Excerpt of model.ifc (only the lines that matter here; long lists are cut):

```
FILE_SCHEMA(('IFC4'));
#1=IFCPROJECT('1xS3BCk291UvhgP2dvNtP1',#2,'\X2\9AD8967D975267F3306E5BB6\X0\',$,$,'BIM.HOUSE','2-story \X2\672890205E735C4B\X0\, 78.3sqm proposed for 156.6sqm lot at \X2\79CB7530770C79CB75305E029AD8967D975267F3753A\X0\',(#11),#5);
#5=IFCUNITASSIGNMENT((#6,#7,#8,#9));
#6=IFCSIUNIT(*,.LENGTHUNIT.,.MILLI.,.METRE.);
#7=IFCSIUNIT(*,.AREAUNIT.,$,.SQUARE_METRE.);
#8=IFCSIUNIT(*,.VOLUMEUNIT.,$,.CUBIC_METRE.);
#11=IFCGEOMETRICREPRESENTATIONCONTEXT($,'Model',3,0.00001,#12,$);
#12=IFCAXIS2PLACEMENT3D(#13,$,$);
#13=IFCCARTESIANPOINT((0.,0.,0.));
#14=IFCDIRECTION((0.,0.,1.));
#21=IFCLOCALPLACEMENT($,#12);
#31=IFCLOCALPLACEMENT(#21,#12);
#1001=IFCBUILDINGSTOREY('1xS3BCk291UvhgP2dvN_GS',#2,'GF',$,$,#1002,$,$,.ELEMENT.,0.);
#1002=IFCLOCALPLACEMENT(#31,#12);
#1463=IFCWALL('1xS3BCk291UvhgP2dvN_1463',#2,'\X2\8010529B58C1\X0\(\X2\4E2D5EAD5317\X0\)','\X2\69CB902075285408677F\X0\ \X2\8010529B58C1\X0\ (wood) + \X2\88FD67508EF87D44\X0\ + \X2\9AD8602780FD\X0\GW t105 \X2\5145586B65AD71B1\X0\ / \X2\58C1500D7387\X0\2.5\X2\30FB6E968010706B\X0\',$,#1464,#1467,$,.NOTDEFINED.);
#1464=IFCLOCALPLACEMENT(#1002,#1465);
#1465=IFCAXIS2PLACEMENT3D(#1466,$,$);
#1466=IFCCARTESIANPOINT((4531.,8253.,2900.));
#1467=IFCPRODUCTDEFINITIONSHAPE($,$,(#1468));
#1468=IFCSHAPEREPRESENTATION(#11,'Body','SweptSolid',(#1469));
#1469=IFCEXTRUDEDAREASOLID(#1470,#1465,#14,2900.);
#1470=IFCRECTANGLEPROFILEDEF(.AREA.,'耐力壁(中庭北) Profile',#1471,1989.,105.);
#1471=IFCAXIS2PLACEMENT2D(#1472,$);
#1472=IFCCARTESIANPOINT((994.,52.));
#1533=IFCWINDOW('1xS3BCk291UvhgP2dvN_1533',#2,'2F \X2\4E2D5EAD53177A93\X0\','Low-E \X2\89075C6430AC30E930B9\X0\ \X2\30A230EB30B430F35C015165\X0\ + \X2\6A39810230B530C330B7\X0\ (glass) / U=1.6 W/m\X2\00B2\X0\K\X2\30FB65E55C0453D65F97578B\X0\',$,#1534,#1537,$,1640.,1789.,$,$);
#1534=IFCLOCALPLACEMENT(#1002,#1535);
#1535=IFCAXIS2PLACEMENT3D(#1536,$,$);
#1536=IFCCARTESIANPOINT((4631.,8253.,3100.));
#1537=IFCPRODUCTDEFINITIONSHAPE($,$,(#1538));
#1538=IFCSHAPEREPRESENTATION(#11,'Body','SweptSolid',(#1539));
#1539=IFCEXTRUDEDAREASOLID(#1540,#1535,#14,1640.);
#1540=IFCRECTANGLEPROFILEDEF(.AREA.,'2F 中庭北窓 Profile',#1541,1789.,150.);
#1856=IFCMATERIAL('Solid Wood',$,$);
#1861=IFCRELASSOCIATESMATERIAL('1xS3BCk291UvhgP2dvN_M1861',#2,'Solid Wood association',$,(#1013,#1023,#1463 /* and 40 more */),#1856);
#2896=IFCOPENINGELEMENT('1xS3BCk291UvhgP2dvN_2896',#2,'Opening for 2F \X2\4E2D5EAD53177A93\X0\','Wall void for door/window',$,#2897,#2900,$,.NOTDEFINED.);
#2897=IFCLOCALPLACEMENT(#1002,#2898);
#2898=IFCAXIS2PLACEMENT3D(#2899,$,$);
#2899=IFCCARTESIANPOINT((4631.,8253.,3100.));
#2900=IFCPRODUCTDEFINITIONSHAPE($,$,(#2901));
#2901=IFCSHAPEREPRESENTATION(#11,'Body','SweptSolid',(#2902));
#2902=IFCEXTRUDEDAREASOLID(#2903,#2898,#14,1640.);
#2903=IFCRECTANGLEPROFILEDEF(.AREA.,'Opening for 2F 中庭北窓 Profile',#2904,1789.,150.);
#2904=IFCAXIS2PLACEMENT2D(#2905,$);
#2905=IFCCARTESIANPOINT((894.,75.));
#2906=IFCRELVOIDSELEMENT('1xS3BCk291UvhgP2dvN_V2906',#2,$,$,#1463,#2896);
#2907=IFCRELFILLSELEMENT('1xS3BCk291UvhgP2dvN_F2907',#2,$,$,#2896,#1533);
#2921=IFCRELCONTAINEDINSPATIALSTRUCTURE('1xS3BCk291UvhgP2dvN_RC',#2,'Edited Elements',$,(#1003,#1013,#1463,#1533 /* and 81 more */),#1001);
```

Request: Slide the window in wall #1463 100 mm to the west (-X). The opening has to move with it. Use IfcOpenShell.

```python
import ifcopenshell
import ifcopenshell.api.geometry
import ifcopenshell.util.placement
import ifcopenshell.util.unit

model = ifcopenshell.open("model.ifc")
unit_scale = ifcopenshell.util.unit.calculate_unit_scale(model)

window = model.by_guid("1xS3BCk291UvhgP2dvN_1533")
opening = window.FillsVoids[0].RelatingOpeningElement
wall = opening.VoidsElements[0].RelatingBuildingElement

wall_matrix = ifcopenshell.util.placement.get_local_placement(wall.ObjectPlacement)
shift = wall_matrix[:3, 0] * -0.1 / unit_scale
before = ifcopenshell.util.placement.get_local_placement(window.ObjectPlacement)[:3, 3].copy()

# The window is not placed relative to its opening, so move both.
for product in (opening, window):
    matrix = ifcopenshell.util.placement.get_local_placement(product.ObjectPlacement)
    matrix[:3, 3] += shift
    ifcopenshell.api.geometry.edit_object_placement(model, product=product, matrix=matrix, is_si=False)

after = ifcopenshell.util.placement.get_local_placement(window.ObjectPlacement)[:3, 3]
print("window moved by", (after - before).round(3) + 0.0)

model.write("model-out.ifc")
```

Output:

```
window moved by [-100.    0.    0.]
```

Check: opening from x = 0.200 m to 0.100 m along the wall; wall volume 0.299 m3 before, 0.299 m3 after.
